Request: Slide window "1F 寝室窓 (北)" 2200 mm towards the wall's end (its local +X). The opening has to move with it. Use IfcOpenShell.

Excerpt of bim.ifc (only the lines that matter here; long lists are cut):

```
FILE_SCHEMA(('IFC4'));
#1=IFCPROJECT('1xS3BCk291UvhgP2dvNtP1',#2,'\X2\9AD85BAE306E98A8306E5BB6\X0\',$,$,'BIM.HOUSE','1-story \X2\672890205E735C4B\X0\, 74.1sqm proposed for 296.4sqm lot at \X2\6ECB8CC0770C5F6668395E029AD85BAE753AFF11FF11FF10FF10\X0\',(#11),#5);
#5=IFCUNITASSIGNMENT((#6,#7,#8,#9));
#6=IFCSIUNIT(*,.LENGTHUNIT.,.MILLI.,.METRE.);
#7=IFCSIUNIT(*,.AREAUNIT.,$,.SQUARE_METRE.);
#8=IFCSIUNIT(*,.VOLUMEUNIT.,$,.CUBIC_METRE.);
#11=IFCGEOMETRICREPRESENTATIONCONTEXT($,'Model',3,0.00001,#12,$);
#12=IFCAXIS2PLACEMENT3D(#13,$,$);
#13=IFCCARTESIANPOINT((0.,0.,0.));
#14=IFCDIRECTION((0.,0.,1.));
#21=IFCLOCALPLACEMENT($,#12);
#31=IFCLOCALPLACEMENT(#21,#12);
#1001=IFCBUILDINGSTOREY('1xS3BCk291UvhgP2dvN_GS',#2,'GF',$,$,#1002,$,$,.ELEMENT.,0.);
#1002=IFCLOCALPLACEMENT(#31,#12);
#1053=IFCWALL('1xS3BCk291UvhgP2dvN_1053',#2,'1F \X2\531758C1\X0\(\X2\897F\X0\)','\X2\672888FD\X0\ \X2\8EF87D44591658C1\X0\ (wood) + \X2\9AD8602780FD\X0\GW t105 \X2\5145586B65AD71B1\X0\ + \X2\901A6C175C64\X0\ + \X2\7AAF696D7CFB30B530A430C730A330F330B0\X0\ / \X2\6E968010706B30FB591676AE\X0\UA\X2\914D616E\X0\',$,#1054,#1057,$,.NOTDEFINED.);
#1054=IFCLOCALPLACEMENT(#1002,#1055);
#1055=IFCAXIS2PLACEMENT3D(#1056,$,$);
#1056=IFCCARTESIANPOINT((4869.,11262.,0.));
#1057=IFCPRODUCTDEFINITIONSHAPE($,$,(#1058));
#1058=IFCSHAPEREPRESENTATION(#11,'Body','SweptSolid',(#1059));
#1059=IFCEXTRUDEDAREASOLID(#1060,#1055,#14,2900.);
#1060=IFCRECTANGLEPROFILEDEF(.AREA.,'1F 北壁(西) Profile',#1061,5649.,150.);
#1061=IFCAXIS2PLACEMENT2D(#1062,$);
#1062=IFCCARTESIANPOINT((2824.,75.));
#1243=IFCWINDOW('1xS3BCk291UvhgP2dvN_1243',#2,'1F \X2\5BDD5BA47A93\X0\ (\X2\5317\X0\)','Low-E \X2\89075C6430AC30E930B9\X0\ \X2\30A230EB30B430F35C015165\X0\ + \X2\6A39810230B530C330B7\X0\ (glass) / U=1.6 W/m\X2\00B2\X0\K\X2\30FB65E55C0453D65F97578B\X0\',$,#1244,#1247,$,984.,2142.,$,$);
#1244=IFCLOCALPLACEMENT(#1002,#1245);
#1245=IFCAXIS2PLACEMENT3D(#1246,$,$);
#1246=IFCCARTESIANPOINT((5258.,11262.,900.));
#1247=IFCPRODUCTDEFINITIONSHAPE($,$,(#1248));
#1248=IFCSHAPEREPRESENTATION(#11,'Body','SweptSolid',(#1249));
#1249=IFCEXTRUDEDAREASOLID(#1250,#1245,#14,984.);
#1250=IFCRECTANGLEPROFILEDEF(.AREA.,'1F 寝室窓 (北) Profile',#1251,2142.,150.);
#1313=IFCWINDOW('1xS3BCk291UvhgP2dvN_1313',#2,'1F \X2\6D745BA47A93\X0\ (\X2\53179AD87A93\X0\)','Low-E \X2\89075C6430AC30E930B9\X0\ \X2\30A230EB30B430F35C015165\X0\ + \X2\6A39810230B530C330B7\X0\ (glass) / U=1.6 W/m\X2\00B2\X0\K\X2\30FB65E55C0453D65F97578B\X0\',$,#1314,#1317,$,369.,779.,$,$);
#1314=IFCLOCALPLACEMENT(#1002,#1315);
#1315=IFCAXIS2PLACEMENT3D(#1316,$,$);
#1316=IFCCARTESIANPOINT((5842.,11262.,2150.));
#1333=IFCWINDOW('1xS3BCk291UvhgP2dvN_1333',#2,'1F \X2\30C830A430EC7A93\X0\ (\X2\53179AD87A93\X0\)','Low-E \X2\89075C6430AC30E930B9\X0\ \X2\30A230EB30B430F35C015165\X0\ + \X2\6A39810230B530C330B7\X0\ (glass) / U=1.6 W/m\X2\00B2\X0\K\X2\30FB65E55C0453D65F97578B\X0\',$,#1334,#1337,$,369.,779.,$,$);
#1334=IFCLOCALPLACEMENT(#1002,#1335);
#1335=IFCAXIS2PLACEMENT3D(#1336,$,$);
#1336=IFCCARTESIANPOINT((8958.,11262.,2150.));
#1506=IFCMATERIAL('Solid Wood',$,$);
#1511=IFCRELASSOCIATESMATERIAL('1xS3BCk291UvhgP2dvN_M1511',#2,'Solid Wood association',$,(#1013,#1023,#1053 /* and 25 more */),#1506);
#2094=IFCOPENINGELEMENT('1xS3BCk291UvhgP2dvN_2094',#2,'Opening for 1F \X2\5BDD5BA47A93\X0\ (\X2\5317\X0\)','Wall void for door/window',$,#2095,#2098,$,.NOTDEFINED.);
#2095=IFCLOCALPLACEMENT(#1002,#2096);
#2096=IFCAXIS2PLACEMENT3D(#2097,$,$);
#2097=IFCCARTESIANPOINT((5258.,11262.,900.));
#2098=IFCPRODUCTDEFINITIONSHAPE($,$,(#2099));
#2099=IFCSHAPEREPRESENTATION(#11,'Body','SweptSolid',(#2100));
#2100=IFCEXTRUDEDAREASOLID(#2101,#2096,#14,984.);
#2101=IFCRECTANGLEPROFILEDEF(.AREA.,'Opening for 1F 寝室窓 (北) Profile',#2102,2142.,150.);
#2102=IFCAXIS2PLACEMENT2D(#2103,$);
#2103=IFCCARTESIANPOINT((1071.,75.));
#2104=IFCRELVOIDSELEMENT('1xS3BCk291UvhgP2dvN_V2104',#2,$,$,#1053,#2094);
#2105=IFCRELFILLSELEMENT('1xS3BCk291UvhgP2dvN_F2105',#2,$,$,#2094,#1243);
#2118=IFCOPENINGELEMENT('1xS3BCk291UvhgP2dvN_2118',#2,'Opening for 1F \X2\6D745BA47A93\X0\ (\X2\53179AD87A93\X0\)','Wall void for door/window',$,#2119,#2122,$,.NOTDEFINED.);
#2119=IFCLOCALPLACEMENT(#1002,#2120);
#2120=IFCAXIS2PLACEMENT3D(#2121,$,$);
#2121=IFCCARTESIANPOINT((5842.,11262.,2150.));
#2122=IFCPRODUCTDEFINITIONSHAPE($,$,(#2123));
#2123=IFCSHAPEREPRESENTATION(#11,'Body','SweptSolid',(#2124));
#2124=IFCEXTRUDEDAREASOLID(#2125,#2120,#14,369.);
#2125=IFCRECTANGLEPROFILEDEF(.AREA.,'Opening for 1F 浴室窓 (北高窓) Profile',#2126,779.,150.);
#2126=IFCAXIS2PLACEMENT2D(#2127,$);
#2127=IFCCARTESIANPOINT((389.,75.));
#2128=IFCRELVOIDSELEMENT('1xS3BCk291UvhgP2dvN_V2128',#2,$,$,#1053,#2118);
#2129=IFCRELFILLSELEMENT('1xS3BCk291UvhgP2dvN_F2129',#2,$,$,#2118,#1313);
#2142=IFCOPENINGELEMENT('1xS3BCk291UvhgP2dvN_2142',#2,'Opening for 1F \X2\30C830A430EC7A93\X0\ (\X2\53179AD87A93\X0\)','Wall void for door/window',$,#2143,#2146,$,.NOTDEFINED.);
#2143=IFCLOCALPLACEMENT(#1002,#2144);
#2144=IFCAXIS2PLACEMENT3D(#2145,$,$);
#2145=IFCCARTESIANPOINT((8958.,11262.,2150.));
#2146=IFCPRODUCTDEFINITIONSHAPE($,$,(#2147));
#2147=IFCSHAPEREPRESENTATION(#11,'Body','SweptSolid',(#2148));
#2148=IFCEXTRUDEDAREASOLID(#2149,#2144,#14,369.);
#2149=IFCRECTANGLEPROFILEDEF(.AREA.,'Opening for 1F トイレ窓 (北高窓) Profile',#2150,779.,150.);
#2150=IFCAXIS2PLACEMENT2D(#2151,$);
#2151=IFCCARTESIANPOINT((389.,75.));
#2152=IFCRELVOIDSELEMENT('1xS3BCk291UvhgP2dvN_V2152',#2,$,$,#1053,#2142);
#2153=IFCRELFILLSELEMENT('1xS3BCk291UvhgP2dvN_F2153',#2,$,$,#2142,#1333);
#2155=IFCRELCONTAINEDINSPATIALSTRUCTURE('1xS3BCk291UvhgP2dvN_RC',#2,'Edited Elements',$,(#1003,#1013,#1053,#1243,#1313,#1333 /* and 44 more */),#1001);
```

```python
import ifcopenshell
import ifcopenshell.api.geometry
import ifcopenshell.util.placement
import ifcopenshell.util.unit

model = ifcopenshell.open("bim.ifc")
unit_scale = ifcopenshell.util.unit.calculate_unit_scale(model)

window = model.by_id(1243)
opening = window.FillsVoids[0].RelatingOpeningElement
wall = opening.VoidsElements[0].RelatingBuildingElement

wall_matrix = ifcopenshell.util.placement.get_local_placement(wall.ObjectPlacement)
shift = wall_matrix[:3, 0] * 2.2 / unit_scale
before = ifcopenshell.util.placement.get_local_placement(window.ObjectPlacement)[:3, 3].copy()

# The window is not placed relative to its opening, so move both.
for product in (opening, window):
    matrix = ifcopenshell.util.placement.get_local_placement(product.ObjectPlacement)
    matrix[:3, 3] += shift
    ifcopenshell.api.geometry.edit_object_placement(model, product=product, matrix=matrix, is_si=False)

after = ifcopenshell.util.placement.get_local_placement(window.ObjectPlacement)[:3, 3]
print("window moved by", (after - before).round(3) + 0.0)

model.write("bim-out.ifc")
```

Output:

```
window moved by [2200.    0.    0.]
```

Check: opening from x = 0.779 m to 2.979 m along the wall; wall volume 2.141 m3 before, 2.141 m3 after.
